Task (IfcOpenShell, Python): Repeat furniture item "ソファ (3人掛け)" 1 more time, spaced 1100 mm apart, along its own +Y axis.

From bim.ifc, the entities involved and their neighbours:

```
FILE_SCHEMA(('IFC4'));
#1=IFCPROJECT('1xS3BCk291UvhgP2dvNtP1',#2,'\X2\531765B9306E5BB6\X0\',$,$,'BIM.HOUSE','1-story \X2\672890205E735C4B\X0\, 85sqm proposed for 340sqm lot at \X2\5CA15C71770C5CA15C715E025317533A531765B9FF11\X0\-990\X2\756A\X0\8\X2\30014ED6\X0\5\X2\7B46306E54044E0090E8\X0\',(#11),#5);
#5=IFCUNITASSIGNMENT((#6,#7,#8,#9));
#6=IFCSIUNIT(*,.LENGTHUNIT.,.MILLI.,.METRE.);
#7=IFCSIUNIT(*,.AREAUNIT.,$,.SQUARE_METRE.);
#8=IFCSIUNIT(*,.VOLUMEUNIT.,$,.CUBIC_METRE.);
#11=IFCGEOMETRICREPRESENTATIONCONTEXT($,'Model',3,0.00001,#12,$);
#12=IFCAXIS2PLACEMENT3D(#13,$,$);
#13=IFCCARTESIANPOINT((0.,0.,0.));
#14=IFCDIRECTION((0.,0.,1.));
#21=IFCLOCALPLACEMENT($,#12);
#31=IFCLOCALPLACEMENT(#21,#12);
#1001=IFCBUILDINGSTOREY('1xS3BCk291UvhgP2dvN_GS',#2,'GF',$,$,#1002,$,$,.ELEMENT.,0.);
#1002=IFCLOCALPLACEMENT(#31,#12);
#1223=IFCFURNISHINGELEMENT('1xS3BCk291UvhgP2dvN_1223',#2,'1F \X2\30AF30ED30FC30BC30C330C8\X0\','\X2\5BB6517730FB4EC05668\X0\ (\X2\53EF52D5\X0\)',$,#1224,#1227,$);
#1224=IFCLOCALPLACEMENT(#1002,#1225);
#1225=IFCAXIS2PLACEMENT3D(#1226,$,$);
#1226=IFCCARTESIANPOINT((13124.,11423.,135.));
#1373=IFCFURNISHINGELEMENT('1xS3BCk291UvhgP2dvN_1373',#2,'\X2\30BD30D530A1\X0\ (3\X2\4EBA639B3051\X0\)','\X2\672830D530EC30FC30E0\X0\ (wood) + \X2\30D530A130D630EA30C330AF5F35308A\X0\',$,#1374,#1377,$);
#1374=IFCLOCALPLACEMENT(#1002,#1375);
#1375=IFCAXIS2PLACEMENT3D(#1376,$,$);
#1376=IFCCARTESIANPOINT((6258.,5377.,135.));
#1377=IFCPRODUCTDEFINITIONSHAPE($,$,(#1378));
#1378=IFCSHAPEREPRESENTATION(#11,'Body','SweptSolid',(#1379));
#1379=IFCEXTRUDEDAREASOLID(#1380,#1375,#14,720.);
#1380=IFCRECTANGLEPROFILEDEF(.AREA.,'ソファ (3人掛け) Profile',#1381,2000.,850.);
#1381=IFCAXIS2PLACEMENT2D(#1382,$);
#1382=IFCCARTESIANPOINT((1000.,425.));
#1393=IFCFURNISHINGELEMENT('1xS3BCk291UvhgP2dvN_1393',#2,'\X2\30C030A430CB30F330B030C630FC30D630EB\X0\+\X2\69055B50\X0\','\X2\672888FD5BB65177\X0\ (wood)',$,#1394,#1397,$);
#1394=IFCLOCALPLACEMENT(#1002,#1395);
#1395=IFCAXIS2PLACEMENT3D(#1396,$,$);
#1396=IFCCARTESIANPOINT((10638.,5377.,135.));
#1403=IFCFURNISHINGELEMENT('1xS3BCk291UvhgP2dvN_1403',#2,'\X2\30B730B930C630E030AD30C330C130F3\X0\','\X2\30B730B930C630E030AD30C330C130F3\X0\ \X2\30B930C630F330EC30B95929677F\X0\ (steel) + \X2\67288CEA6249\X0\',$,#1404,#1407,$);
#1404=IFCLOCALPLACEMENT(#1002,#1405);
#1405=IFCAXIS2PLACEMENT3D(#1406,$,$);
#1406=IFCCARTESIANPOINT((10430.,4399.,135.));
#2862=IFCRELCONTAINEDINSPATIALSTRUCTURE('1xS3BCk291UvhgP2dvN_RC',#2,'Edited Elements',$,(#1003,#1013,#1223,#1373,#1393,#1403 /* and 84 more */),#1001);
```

```python
import ifcopenshell
import ifcopenshell.api.geometry
import ifcopenshell.api.root
import ifcopenshell.util.element
import ifcopenshell.util.placement
import ifcopenshell.util.unit

model = ifcopenshell.open("bim.ifc")
unit_scale = ifcopenshell.util.unit.calculate_unit_scale(model)


def reuse_history(source, copy):
    """copy_class also copies each property set's owner history, people and application; keep the originals."""
    for rel in copy.IsDefinedBy:
        if rel.is_a("IfcRelDefinesByProperties") and (history := rel.RelatingPropertyDefinition.OwnerHistory):
            rel.RelatingPropertyDefinition.OwnerHistory = source.OwnerHistory
            ifcopenshell.util.element.remove_deep2(model, history)


source = model.by_guid("1xS3BCk291UvhgP2dvN_1373")
base = ifcopenshell.util.placement.get_local_placement(source.ObjectPlacement)
step = base[:3, 1] * 1.1 / unit_scale

for i in range(1, 2):
    copy = ifcopenshell.api.root.copy_class(model, product=source)
    copy.Representation = ifcopenshell.util.element.copy_deep(
        model, source.Representation, exclude=["IfcGeometricRepresentationContext", "IfcRepresentationMap"]
    )
    reuse_history(source, copy)
    matrix = base.copy()
    matrix[:3, 3] += i * step
    print("added at", matrix[:3, 3].round(3) + 0.0)
    ifcopenshell.api.geometry.edit_object_placement(model, product=copy, matrix=matrix, is_si=False)

model.write("bim_v2.ifc")
```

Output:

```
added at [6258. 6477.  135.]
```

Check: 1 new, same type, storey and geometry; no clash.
